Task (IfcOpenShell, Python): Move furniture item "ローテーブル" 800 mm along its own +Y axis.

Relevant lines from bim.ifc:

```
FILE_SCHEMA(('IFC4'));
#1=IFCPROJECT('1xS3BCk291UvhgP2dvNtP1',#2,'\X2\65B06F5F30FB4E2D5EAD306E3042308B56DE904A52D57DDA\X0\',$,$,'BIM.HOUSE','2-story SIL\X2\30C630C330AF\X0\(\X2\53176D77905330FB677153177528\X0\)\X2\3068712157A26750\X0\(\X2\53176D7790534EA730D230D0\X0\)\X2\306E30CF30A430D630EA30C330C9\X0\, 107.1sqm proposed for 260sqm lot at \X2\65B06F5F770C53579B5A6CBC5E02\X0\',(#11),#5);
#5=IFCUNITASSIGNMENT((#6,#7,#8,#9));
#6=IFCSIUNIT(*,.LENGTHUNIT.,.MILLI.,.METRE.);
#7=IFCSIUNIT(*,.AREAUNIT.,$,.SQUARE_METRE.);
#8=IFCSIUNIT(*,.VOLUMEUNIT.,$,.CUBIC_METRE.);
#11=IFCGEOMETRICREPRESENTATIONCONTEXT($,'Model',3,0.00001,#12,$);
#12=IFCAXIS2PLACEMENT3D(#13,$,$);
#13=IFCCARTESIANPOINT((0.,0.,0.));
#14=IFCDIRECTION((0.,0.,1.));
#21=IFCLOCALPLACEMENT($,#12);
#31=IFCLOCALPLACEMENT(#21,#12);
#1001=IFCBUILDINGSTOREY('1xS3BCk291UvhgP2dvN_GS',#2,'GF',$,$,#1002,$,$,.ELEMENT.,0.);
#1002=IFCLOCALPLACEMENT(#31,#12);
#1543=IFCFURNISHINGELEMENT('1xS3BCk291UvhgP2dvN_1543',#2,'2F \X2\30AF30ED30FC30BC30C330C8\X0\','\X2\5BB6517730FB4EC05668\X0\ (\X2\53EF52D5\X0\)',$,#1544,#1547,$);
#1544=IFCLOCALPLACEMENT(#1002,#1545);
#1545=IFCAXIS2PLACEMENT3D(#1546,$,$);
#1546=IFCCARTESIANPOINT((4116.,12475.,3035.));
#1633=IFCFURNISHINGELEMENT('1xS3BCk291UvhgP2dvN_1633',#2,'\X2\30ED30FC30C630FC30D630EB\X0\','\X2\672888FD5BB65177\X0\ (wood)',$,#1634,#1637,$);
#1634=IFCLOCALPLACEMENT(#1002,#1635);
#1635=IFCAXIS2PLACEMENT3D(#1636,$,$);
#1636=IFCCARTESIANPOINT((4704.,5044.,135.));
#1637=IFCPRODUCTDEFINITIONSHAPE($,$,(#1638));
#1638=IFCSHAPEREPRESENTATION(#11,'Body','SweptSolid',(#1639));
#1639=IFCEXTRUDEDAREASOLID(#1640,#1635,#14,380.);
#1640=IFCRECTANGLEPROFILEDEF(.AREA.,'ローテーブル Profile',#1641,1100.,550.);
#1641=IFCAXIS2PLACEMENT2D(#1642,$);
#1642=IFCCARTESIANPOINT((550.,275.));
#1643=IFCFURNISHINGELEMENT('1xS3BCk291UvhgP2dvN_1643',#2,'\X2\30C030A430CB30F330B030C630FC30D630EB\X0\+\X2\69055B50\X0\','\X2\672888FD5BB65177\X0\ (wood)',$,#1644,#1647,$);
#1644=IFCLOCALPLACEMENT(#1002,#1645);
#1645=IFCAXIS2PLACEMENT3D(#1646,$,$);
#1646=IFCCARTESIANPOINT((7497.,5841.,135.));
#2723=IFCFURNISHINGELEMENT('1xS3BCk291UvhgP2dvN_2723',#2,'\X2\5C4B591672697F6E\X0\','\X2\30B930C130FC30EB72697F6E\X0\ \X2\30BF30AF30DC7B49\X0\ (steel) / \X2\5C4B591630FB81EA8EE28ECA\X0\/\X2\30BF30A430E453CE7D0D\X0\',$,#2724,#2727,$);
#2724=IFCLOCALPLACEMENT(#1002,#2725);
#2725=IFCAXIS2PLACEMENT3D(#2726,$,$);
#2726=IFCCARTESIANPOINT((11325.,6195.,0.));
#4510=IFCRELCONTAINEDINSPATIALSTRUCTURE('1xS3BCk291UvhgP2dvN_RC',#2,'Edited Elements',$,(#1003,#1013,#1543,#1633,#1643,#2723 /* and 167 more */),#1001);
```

```python
import ifcopenshell
import ifcopenshell.api.geometry
import ifcopenshell.util.placement
import ifcopenshell.util.unit

model = ifcopenshell.open("bim.ifc")
unit_scale = ifcopenshell.util.unit.calculate_unit_scale(model)

item = model.by_guid("1xS3BCk291UvhgP2dvN_1633")
matrix = ifcopenshell.util.placement.get_local_placement(item.ObjectPlacement)
matrix[:3, 3] += matrix[:3, 1] * 0.8 / unit_scale
ifcopenshell.api.geometry.edit_object_placement(model, product=item, matrix=matrix, is_si=False)

print(ifcopenshell.util.placement.get_local_placement(item.ObjectPlacement).round(3) + 0.0)

model.write("bim_updated.ifc")
```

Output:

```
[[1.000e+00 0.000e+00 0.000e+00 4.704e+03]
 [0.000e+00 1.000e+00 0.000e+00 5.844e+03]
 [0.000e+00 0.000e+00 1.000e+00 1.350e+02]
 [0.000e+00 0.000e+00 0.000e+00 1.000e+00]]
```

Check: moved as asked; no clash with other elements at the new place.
